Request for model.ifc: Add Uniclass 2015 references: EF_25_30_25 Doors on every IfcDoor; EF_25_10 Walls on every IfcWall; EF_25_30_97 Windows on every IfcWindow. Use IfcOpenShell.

First a look at what the model holds.

```python
import ifcopenshell

model = ifcopenshell.open("model.ifc")
print(model.schema)
print("classifications:", [c.Name for c in model.by_type("IfcClassification")])
for ifc_class in ("IfcDoor", "IfcRoof", "IfcStair", "IfcWall", "IfcWindow"):
    print(ifc_class, len(model.by_type(ifc_class)))
```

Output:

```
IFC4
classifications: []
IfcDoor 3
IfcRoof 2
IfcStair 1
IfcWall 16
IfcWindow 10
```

```python
import ifcopenshell
import ifcopenshell.api.classification

model = ifcopenshell.open("model.ifc")

system = ifcopenshell.api.classification.add_classification(model, classification="Uniclass 2015")

codes = {
    "IfcDoor": ("EF_25_30_25", "Doors"),
    "IfcWall": ("EF_25_10", "Walls"),
    "IfcWindow": ("EF_25_30_97", "Windows"),
}
for ifc_class, (code, name) in codes.items():
    products = model.by_type(ifc_class)
    ifcopenshell.api.classification.add_reference(
        model, products=products, classification=system, identification=code, name=name
    )
    print(code, len(products))

model.write("model_edited.ifc")
```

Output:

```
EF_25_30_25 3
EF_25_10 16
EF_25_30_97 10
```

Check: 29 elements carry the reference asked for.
